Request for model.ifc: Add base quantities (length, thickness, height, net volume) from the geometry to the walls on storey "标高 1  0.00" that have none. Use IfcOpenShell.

First a look at what the model holds.

```python
import ifcopenshell
import ifcopenshell.util.element
import ifcopenshell.util.unit

model = ifcopenshell.open("model.ifc")
print(model.schema)
for unit_type in ("LENGTHUNIT", "AREAUNIT", "VOLUMEUNIT"):
    print(unit_type, ifcopenshell.util.unit.calculate_unit_scale(model, unit_type))
storey = next(s for s in model.by_type("IfcBuildingStorey") if s.Name == "标高 1  0.00")
walls = [e for e in ifcopenshell.util.element.get_decomposition(storey) if e.is_a("IfcWall")]
for e in sorted(walls, key=lambda e: e.id()):
    print(e.id(), e.is_a(), e.Name, list(ifcopenshell.util.element.get_psets(e, qtos_only=True)), sep=" | ")
```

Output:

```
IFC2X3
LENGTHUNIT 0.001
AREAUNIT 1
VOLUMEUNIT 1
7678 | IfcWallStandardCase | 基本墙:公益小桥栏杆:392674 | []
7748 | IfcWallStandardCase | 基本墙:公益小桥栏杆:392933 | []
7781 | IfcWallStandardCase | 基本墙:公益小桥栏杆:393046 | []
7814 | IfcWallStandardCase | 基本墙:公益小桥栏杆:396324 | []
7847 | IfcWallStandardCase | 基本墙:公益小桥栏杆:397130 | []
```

```python
import ifcopenshell
import ifcopenshell.api.pset
import ifcopenshell.geom
import ifcopenshell.util.element
import ifcopenshell.util.shape
import ifcopenshell.util.unit

model = ifcopenshell.open("model.ifc")
unit_scale = ifcopenshell.util.unit.calculate_unit_scale(model)
volume_scale = ifcopenshell.util.unit.calculate_unit_scale(model, "VOLUMEUNIT")
settings = ifcopenshell.geom.settings()

storey = next(s for s in model.by_type("IfcBuildingStorey") if s.Name == "标高 1  0.00")
walls = [e for e in ifcopenshell.util.element.get_decomposition(storey) if e.is_a("IfcWall")]

for e in sorted(walls, key=lambda e: e.id()):
    if ifcopenshell.util.element.get_psets(e, qtos_only=True, should_inherit=False):
        continue
    # Geometry comes back in metres, in the element's own axes.
    shape = ifcopenshell.geom.create_shape(settings, e)
    values = {
        "Length": ifcopenshell.util.shape.get_x(shape.geometry) / unit_scale,
        "Width": ifcopenshell.util.shape.get_y(shape.geometry) / unit_scale,
        "Height": ifcopenshell.util.shape.get_z(shape.geometry) / unit_scale,
        "NetVolume": ifcopenshell.util.shape.get_volume(shape.geometry) / volume_scale,
    }
    qto = ifcopenshell.api.pset.add_qto(model, product=e, name="BaseQuantities")
    ifcopenshell.api.pset.edit_qto(model, qto=qto, properties=values)
    print(e.id(), {k: round(v, 3) for k, v in values.items()})

model.write("model_updated.ifc")
```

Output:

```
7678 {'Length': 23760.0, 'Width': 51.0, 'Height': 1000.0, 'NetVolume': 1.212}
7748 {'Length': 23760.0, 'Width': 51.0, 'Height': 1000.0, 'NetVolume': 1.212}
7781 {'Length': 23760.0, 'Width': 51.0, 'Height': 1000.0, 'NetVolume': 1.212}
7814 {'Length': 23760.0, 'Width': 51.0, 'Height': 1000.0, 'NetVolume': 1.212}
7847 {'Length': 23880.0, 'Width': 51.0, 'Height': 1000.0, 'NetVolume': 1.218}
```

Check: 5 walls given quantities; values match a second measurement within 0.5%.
